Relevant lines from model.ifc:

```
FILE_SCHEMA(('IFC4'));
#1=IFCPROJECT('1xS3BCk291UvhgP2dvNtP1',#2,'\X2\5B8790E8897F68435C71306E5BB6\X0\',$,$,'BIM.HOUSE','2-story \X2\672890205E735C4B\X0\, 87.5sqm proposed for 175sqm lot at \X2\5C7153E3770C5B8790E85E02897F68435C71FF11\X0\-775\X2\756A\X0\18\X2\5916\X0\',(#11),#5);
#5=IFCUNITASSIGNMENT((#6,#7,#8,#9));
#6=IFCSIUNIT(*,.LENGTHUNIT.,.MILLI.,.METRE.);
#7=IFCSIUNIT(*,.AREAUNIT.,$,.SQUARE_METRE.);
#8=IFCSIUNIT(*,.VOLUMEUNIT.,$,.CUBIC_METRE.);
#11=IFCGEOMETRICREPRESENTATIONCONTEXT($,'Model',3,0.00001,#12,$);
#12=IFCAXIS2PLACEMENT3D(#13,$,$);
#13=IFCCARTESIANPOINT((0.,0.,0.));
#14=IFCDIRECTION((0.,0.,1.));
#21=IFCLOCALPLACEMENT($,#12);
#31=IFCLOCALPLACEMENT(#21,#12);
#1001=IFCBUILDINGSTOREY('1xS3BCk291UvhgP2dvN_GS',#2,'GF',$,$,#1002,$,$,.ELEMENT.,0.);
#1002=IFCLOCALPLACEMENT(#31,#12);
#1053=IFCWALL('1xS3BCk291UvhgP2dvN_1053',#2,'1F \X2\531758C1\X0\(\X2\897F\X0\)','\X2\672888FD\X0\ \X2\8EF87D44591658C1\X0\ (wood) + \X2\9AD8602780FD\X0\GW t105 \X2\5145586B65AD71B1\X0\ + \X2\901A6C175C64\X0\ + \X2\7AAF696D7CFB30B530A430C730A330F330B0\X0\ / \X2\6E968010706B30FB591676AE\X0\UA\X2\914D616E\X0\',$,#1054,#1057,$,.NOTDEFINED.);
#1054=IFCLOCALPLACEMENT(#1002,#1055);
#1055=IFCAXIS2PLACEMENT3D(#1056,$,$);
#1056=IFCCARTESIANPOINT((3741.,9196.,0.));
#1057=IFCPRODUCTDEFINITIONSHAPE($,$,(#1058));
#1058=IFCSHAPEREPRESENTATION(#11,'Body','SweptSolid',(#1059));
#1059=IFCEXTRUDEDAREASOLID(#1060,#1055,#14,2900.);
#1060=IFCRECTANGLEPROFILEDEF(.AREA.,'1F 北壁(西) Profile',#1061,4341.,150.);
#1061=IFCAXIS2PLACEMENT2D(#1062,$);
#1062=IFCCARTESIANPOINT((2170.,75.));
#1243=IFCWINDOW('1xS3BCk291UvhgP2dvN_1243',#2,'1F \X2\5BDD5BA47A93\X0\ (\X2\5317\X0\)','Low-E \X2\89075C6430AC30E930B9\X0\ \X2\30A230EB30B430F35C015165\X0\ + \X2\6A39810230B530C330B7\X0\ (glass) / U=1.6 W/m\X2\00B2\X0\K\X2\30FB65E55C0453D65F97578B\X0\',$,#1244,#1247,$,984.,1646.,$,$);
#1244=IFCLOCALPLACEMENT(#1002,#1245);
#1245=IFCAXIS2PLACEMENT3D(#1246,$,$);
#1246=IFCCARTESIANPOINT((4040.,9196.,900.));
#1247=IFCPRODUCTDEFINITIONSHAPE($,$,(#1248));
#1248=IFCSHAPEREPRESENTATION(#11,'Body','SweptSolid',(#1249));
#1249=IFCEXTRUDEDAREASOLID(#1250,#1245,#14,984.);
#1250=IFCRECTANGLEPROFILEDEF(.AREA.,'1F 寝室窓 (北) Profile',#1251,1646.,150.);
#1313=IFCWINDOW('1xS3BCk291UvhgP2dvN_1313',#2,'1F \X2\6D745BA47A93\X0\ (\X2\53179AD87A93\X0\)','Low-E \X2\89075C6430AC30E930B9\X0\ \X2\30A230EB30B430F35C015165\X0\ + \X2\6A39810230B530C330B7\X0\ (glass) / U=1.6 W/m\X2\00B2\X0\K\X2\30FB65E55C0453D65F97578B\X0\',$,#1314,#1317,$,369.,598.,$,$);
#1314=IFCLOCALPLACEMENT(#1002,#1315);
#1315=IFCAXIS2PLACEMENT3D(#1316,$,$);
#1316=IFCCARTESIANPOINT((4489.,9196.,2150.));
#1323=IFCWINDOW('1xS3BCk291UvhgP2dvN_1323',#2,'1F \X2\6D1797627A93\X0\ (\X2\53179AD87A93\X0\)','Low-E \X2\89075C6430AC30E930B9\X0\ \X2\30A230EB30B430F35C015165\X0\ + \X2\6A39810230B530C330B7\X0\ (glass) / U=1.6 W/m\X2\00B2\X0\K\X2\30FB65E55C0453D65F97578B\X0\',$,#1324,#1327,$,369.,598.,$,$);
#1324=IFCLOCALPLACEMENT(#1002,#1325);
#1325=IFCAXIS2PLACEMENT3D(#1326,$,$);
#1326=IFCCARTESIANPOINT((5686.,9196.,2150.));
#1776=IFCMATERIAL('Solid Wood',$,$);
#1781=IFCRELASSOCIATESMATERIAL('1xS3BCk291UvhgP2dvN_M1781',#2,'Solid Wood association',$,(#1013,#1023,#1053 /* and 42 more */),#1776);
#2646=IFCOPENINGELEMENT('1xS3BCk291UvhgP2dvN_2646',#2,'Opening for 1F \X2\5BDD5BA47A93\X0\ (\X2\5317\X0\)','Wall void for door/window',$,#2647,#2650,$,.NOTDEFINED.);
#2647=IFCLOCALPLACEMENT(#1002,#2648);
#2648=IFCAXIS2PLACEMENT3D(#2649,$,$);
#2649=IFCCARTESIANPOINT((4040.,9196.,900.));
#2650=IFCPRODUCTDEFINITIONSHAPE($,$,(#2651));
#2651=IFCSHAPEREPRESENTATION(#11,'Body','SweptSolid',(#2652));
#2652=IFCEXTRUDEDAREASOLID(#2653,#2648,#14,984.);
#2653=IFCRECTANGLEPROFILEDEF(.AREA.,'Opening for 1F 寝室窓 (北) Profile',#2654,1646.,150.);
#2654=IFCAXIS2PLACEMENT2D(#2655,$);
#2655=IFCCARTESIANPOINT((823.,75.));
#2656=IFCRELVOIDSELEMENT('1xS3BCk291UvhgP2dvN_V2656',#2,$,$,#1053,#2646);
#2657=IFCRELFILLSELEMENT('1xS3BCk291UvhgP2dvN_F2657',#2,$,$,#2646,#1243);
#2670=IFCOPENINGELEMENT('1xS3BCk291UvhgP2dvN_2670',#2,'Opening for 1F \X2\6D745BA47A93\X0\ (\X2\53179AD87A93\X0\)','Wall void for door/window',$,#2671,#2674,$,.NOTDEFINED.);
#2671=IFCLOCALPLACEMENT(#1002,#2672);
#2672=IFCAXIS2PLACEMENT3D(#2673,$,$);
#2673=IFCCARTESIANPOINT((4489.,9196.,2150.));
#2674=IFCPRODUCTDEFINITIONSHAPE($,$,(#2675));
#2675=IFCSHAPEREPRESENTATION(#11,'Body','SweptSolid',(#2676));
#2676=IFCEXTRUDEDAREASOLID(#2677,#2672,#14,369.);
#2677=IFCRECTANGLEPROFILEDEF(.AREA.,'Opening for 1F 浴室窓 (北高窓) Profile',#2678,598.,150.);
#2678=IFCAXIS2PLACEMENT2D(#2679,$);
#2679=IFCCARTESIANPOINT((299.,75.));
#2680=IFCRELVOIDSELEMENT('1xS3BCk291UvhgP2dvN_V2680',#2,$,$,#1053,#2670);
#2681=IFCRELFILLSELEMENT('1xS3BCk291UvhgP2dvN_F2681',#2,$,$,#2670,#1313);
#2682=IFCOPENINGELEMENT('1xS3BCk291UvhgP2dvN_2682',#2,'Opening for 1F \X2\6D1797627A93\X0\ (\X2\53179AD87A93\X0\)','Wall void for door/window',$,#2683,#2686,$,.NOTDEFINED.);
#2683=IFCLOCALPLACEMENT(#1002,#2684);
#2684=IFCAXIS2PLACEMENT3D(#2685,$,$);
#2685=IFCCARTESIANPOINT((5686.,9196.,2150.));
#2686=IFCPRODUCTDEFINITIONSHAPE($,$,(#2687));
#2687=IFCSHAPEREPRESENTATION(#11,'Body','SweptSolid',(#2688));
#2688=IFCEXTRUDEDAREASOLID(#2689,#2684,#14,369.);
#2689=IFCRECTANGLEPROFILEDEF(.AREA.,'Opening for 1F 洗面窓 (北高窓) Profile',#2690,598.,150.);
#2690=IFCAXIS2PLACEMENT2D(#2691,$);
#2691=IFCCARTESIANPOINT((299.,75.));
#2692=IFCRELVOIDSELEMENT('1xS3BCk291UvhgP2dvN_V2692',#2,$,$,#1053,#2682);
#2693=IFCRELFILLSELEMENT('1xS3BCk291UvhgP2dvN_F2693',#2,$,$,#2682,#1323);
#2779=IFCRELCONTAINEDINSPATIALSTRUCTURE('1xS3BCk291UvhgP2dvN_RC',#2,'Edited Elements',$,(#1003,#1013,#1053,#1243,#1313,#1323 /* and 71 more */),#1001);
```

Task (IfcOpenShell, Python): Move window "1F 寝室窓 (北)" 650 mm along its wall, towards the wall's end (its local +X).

```python
import ifcopenshell
import ifcopenshell.api.geometry
import ifcopenshell.util.placement

model = ifcopenshell.open("model.ifc")

window = model.by_guid("1xS3BCk291UvhgP2dvN_1243")
opening = window.FillsVoids[0].RelatingOpeningElement
wall = opening.VoidsElements[0].RelatingBuildingElement

wall_matrix = ifcopenshell.util.placement.get_local_placement(wall.ObjectPlacement)
shift = wall_matrix[:3, 0] * 650.0
before = ifcopenshell.util.placement.get_local_placement(window.ObjectPlacement)[:3, 3].copy()

# The window is not placed relative to its opening, so move both.
for product in (opening, window):
    matrix = ifcopenshell.util.placement.get_local_placement(product.ObjectPlacement)
    matrix[:3, 3] += shift
    ifcopenshell.api.geometry.edit_object_placement(model, product=product, matrix=matrix, is_si=False)

after = ifcopenshell.util.placement.get_local_placement(window.ObjectPlacement)[:3, 3]
print("window moved by", (after - before).round(3) + 0.0)

model.write("model_v2.ifc")
```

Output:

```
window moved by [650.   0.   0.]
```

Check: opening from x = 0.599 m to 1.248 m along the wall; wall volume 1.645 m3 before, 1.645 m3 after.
